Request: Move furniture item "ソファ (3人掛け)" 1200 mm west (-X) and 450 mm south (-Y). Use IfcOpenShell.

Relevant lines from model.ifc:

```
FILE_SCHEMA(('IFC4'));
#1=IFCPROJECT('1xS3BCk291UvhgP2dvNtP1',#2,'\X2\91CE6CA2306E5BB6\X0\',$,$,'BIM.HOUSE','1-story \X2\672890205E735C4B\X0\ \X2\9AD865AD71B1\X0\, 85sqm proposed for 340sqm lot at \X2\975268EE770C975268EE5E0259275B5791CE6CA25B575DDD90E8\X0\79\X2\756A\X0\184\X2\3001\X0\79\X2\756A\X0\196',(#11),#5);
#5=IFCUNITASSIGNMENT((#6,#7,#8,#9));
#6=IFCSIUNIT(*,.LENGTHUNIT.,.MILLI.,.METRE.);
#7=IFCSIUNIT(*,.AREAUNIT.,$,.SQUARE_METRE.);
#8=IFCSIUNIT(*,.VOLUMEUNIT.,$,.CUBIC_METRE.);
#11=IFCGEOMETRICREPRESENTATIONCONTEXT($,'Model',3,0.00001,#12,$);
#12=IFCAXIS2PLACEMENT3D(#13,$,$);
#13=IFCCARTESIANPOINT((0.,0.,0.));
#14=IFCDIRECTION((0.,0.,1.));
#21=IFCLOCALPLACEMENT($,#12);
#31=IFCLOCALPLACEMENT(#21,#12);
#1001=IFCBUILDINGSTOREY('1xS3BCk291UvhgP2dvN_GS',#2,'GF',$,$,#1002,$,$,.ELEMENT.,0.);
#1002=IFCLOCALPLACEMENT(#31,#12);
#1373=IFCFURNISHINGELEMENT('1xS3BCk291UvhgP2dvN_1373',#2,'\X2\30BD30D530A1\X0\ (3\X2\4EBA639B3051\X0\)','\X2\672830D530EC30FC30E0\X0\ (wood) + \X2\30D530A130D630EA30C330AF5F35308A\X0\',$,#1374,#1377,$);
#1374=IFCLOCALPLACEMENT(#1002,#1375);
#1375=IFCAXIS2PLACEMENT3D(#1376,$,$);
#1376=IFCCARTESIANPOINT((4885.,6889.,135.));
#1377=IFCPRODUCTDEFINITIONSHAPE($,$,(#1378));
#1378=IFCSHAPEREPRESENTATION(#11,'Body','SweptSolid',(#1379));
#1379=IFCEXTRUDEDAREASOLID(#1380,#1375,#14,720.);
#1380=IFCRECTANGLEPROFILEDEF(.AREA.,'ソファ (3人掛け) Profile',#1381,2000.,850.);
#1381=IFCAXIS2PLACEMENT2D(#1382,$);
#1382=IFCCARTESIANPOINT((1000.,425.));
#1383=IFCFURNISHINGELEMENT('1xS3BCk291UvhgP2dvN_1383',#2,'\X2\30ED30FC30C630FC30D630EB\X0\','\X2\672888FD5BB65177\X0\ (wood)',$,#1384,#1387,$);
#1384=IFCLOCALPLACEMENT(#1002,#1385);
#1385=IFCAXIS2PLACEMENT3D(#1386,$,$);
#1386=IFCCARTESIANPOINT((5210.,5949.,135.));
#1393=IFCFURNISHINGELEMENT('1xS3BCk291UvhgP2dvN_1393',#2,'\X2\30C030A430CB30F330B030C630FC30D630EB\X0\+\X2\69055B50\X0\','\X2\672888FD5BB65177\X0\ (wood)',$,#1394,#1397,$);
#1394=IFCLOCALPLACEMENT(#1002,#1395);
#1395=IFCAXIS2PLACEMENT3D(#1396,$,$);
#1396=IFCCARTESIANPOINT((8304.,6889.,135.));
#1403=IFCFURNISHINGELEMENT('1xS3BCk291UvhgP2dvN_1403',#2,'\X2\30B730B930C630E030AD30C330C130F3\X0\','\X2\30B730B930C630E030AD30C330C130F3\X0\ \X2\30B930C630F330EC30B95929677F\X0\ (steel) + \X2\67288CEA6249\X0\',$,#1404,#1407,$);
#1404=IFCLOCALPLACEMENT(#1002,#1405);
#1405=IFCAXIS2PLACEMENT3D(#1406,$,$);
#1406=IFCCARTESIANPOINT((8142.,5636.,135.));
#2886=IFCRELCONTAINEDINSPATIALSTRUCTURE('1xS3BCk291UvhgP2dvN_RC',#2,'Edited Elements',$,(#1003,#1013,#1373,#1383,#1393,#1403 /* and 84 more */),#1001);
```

```python
import ifcopenshell
import ifcopenshell.api.geometry
import ifcopenshell.util.placement
import ifcopenshell.util.unit

model = ifcopenshell.open("model.ifc")
unit_scale = ifcopenshell.util.unit.calculate_unit_scale(model)

item = model.by_guid("1xS3BCk291UvhgP2dvN_1373")
matrix = ifcopenshell.util.placement.get_local_placement(item.ObjectPlacement)
matrix[0, 3] -= 1.2 / unit_scale
matrix[1, 3] -= 0.45 / unit_scale
ifcopenshell.api.geometry.edit_object_placement(model, product=item, matrix=matrix, is_si=False)

print(ifcopenshell.util.placement.get_local_placement(item.ObjectPlacement).round(3) + 0.0)

model.write("model_v2.ifc")
```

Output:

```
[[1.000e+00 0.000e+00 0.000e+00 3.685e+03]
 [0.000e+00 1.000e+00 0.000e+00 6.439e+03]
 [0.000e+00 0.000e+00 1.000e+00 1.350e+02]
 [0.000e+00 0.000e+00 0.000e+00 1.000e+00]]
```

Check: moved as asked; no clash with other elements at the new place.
